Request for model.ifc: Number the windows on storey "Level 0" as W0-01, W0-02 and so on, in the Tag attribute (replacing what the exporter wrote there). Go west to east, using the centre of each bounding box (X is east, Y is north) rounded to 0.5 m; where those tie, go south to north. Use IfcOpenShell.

First a look at what the model holds.

```python
import ifcopenshell
import ifcopenshell.util.element
import ifcopenshell.util.placement

model = ifcopenshell.open("model.ifc")
print(model.schema)
storey = next(s for s in model.by_type("IfcBuildingStorey") if s.Name == "Level 0")
windows = [e for e in ifcopenshell.util.element.get_decomposition(storey) if e.is_a("IfcWindow")]
for e in sorted(windows, key=lambda e: e.id()):
    origin = ifcopenshell.util.placement.get_local_placement(e.ObjectPlacement)[:3, 3]
    print(e.id(), e.Tag, e.Name, origin.round(2) + 0.0, sep=" | ")
```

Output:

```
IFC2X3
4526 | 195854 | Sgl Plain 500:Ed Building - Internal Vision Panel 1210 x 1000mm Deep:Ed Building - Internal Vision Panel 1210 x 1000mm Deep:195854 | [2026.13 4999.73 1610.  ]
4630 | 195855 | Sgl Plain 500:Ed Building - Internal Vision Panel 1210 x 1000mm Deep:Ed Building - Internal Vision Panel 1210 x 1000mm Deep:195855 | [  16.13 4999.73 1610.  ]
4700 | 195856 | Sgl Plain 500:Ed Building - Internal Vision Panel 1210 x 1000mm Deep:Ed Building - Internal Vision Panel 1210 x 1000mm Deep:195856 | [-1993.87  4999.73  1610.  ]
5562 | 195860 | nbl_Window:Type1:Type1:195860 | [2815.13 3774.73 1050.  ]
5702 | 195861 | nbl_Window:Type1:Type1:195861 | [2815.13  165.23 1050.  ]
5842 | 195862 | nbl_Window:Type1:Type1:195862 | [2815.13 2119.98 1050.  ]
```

```python
import ifcopenshell
import ifcopenshell.geom
import ifcopenshell.util.element
import ifcopenshell.util.shape

model = ifcopenshell.open("model.ifc")
settings = ifcopenshell.geom.settings()
settings.set("use-world-coords", True)


def centre(element):
    shape = ifcopenshell.geom.create_shape(settings, element)
    return ifcopenshell.util.shape.get_bbox_centroid(shape.geometry)


storey = next(s for s in model.by_type("IfcBuildingStorey") if s.Name == "Level 0")
windows = [e for e in ifcopenshell.util.element.get_decomposition(storey) if e.is_a("IfcWindow")]

# Insertion points can sit at a corner or the storey origin, so sort by the geometry (in metres).
centres = {e: centre(e) for e in windows}
windows.sort(key=lambda e: (round(centres[e][0] / 0.5), centres[e][1]))

for i, e in enumerate(windows, start=1):
    number = f"W0-{i:02d}"
    e.Tag = number
    print(e.id(), number)

model.write("model_updated.ifc")
```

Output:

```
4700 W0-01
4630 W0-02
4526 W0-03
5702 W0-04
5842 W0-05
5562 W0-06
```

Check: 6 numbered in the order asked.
